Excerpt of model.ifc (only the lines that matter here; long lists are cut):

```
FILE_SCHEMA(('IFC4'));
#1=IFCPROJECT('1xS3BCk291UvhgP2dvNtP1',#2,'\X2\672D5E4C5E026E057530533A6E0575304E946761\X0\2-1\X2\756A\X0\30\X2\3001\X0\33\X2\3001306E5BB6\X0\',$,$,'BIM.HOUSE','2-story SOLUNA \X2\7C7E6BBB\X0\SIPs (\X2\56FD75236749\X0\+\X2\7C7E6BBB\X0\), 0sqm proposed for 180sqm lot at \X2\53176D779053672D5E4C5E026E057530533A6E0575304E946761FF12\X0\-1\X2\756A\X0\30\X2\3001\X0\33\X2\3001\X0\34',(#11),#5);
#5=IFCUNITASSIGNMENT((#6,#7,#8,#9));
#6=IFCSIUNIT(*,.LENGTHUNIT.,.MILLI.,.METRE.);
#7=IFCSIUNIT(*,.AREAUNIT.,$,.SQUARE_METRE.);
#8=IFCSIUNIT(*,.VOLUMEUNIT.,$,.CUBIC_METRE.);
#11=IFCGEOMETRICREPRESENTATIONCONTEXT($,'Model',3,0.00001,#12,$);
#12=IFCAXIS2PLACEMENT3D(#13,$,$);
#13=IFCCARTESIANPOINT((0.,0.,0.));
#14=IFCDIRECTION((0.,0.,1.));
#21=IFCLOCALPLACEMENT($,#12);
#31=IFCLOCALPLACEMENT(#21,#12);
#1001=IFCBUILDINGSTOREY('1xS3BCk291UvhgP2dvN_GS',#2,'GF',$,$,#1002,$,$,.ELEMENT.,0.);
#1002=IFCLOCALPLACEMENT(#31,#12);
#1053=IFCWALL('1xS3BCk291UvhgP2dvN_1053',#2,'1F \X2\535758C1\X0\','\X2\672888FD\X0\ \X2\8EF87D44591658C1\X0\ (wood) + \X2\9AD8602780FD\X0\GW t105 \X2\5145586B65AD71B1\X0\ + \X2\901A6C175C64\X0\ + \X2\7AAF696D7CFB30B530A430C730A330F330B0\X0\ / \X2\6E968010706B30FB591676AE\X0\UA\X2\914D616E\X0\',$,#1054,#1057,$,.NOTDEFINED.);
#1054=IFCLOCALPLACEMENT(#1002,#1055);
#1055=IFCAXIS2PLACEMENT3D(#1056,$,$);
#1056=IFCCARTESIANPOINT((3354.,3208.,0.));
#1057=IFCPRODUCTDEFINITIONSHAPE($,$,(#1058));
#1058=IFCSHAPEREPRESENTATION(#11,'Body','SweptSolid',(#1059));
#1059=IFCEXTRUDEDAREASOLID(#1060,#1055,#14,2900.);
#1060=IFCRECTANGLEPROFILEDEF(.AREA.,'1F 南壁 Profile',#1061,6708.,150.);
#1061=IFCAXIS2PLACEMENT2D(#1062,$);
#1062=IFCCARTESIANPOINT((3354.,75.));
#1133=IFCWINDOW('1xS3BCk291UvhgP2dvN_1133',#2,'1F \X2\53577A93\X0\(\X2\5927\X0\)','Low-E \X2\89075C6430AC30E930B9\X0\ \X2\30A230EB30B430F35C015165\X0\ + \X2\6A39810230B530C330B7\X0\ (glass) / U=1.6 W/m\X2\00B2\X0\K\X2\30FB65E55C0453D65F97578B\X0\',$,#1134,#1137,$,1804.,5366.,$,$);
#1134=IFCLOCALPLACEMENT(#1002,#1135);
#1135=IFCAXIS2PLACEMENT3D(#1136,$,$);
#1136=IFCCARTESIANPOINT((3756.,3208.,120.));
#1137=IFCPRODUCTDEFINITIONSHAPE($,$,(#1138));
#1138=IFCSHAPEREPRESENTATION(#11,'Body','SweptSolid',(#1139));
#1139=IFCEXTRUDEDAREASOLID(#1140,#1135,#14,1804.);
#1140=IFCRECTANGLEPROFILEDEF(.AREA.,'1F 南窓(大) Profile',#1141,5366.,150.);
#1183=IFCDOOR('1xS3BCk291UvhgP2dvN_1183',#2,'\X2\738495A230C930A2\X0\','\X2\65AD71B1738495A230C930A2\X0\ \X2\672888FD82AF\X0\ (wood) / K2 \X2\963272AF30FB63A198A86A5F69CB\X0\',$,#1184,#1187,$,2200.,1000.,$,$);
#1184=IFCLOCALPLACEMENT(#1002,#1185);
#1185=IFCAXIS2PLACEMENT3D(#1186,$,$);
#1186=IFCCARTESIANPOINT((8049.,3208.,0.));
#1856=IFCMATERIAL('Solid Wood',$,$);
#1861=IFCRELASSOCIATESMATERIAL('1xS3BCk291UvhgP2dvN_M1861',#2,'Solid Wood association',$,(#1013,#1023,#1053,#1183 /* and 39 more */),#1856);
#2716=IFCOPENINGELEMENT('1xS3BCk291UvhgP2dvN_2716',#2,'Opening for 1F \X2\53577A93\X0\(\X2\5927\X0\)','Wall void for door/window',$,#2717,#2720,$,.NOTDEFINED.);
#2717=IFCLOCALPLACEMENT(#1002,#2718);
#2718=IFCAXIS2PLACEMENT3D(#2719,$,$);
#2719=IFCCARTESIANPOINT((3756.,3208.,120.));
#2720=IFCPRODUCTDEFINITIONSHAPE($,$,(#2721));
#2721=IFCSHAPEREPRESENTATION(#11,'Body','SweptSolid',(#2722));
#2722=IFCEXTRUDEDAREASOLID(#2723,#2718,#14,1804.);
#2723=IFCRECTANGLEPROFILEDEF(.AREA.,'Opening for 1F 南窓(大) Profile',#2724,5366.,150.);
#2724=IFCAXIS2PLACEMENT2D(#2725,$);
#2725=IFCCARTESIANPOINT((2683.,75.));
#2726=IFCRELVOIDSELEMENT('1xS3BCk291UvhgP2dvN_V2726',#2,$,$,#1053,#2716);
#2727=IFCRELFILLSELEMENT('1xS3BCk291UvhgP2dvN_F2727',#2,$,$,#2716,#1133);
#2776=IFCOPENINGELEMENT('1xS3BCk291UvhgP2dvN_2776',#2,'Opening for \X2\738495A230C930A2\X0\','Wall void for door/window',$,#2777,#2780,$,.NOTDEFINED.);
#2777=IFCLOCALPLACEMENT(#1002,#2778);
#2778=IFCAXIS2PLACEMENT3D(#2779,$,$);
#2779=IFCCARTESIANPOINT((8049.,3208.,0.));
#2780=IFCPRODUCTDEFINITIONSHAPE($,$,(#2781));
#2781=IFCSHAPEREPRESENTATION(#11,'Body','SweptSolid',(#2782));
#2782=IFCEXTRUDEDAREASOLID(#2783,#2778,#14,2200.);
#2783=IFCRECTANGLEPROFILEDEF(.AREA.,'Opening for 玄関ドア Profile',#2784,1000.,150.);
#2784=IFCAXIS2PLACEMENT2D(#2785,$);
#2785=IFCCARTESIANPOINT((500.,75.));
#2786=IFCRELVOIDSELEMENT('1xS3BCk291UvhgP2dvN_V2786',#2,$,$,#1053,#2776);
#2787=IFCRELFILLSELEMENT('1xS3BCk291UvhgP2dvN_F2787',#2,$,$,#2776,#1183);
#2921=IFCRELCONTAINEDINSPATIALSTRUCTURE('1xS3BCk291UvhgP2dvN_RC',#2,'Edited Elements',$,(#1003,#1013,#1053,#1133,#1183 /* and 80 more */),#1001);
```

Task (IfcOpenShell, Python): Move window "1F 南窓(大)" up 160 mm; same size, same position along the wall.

```python
import numpy as np
import ifcopenshell
import ifcopenshell.api.geometry
import ifcopenshell.util.placement
import ifcopenshell.util.unit

model = ifcopenshell.open("model.ifc")
unit_scale = ifcopenshell.util.unit.calculate_unit_scale(model)

window = model.by_guid("1xS3BCk291UvhgP2dvN_1133")
opening = window.FillsVoids[0].RelatingOpeningElement
dz = 0.16 / unit_scale

shift = np.array([0.0, 0.0, dz])
# The window is not placed relative to its opening, so move both.
for product in (opening, window):
    matrix = ifcopenshell.util.placement.get_local_placement(product.ObjectPlacement)
    matrix[:3, 3] += shift
    ifcopenshell.api.geometry.edit_object_placement(model, product=product, matrix=matrix, is_si=False)

print(f"moved by {dz * unit_scale:+.3f} m")

model.write("model_updated.ifc")
```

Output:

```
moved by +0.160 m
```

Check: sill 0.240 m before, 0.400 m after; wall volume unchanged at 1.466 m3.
